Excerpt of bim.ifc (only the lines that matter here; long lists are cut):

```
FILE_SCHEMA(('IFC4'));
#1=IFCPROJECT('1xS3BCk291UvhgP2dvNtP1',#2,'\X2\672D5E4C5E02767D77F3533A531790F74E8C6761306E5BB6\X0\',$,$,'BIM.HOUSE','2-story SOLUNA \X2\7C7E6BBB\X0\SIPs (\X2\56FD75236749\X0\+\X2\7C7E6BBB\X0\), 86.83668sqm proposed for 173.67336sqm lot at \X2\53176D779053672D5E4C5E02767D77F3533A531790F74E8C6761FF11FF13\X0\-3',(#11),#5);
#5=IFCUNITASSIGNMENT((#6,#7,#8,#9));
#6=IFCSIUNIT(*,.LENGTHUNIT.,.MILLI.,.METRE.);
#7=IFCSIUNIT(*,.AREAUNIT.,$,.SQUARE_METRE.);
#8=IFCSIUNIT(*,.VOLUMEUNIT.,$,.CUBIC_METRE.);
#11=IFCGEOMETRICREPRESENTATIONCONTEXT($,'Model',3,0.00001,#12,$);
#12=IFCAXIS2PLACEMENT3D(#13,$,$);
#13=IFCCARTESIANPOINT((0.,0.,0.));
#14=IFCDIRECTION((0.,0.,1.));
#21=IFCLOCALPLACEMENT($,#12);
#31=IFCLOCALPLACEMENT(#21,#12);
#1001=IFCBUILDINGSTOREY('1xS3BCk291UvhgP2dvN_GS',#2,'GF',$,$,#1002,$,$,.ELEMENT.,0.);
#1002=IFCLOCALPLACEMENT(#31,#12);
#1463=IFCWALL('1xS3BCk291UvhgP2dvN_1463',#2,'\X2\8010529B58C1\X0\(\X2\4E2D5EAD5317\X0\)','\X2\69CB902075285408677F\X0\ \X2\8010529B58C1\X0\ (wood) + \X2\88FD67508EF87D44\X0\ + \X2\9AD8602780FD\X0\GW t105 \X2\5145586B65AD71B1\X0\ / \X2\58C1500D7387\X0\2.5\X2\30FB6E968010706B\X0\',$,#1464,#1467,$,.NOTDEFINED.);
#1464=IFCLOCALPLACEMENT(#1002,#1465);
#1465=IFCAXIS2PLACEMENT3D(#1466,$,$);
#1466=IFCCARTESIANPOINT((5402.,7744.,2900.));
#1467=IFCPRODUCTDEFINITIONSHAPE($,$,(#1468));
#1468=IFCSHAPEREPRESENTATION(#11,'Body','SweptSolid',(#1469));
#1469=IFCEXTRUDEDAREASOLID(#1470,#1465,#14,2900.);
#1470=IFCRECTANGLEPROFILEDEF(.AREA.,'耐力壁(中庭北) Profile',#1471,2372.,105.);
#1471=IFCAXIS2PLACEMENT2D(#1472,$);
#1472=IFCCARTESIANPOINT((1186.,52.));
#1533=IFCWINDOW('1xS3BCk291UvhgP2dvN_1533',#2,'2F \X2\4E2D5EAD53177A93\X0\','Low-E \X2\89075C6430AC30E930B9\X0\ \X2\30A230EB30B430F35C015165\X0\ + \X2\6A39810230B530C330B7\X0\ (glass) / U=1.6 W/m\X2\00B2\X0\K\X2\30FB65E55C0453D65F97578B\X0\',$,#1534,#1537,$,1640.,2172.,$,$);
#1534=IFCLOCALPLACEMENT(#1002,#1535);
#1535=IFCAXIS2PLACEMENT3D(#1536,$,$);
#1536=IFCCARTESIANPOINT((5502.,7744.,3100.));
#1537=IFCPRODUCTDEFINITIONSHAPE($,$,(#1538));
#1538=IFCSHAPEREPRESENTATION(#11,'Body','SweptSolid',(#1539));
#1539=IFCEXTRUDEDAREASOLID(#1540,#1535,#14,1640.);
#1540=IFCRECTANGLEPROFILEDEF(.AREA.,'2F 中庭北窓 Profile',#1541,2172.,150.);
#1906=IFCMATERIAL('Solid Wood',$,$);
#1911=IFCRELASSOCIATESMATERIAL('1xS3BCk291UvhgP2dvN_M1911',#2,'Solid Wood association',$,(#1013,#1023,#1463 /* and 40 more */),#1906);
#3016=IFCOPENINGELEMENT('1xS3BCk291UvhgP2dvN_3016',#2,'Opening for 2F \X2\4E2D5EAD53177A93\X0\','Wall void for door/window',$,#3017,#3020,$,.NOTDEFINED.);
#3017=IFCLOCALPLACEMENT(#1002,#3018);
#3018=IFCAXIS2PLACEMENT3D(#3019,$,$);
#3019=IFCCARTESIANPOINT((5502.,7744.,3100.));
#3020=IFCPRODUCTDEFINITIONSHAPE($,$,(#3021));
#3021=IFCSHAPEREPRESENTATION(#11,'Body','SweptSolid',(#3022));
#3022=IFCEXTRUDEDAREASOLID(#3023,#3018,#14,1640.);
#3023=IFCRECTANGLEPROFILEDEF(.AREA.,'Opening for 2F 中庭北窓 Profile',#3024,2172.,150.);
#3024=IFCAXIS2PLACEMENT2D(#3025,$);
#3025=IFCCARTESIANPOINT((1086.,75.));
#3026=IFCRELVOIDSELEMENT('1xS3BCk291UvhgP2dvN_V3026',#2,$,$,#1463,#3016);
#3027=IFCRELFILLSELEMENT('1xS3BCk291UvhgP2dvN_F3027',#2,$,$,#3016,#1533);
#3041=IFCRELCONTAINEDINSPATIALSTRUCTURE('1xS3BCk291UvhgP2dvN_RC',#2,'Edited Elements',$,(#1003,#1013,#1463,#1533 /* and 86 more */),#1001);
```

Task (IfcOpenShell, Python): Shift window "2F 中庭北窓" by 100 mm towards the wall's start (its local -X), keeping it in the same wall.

```python
import ifcopenshell
import ifcopenshell.api.geometry
import ifcopenshell.util.placement
import ifcopenshell.util.unit

model = ifcopenshell.open("bim.ifc")
unit_scale = ifcopenshell.util.unit.calculate_unit_scale(model)

window = model.by_guid("1xS3BCk291UvhgP2dvN_1533")
opening = window.FillsVoids[0].RelatingOpeningElement
wall = opening.VoidsElements[0].RelatingBuildingElement

wall_matrix = ifcopenshell.util.placement.get_local_placement(wall.ObjectPlacement)
shift = wall_matrix[:3, 0] * -0.1 / unit_scale
before = ifcopenshell.util.placement.get_local_placement(window.ObjectPlacement)[:3, 3].copy()

# The window is not placed relative to its opening, so move both.
for product in (opening, window):
    matrix = ifcopenshell.util.placement.get_local_placement(product.ObjectPlacement)
    matrix[:3, 3] += shift
    ifcopenshell.api.geometry.edit_object_placement(model, product=product, matrix=matrix, is_si=False)

after = ifcopenshell.util.placement.get_local_placement(window.ObjectPlacement)[:3, 3]
print("window moved by", (after - before).round(3) + 0.0)

model.write("bim_edited.ifc")
```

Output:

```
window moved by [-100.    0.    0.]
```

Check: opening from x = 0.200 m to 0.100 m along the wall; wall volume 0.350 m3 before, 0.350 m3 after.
